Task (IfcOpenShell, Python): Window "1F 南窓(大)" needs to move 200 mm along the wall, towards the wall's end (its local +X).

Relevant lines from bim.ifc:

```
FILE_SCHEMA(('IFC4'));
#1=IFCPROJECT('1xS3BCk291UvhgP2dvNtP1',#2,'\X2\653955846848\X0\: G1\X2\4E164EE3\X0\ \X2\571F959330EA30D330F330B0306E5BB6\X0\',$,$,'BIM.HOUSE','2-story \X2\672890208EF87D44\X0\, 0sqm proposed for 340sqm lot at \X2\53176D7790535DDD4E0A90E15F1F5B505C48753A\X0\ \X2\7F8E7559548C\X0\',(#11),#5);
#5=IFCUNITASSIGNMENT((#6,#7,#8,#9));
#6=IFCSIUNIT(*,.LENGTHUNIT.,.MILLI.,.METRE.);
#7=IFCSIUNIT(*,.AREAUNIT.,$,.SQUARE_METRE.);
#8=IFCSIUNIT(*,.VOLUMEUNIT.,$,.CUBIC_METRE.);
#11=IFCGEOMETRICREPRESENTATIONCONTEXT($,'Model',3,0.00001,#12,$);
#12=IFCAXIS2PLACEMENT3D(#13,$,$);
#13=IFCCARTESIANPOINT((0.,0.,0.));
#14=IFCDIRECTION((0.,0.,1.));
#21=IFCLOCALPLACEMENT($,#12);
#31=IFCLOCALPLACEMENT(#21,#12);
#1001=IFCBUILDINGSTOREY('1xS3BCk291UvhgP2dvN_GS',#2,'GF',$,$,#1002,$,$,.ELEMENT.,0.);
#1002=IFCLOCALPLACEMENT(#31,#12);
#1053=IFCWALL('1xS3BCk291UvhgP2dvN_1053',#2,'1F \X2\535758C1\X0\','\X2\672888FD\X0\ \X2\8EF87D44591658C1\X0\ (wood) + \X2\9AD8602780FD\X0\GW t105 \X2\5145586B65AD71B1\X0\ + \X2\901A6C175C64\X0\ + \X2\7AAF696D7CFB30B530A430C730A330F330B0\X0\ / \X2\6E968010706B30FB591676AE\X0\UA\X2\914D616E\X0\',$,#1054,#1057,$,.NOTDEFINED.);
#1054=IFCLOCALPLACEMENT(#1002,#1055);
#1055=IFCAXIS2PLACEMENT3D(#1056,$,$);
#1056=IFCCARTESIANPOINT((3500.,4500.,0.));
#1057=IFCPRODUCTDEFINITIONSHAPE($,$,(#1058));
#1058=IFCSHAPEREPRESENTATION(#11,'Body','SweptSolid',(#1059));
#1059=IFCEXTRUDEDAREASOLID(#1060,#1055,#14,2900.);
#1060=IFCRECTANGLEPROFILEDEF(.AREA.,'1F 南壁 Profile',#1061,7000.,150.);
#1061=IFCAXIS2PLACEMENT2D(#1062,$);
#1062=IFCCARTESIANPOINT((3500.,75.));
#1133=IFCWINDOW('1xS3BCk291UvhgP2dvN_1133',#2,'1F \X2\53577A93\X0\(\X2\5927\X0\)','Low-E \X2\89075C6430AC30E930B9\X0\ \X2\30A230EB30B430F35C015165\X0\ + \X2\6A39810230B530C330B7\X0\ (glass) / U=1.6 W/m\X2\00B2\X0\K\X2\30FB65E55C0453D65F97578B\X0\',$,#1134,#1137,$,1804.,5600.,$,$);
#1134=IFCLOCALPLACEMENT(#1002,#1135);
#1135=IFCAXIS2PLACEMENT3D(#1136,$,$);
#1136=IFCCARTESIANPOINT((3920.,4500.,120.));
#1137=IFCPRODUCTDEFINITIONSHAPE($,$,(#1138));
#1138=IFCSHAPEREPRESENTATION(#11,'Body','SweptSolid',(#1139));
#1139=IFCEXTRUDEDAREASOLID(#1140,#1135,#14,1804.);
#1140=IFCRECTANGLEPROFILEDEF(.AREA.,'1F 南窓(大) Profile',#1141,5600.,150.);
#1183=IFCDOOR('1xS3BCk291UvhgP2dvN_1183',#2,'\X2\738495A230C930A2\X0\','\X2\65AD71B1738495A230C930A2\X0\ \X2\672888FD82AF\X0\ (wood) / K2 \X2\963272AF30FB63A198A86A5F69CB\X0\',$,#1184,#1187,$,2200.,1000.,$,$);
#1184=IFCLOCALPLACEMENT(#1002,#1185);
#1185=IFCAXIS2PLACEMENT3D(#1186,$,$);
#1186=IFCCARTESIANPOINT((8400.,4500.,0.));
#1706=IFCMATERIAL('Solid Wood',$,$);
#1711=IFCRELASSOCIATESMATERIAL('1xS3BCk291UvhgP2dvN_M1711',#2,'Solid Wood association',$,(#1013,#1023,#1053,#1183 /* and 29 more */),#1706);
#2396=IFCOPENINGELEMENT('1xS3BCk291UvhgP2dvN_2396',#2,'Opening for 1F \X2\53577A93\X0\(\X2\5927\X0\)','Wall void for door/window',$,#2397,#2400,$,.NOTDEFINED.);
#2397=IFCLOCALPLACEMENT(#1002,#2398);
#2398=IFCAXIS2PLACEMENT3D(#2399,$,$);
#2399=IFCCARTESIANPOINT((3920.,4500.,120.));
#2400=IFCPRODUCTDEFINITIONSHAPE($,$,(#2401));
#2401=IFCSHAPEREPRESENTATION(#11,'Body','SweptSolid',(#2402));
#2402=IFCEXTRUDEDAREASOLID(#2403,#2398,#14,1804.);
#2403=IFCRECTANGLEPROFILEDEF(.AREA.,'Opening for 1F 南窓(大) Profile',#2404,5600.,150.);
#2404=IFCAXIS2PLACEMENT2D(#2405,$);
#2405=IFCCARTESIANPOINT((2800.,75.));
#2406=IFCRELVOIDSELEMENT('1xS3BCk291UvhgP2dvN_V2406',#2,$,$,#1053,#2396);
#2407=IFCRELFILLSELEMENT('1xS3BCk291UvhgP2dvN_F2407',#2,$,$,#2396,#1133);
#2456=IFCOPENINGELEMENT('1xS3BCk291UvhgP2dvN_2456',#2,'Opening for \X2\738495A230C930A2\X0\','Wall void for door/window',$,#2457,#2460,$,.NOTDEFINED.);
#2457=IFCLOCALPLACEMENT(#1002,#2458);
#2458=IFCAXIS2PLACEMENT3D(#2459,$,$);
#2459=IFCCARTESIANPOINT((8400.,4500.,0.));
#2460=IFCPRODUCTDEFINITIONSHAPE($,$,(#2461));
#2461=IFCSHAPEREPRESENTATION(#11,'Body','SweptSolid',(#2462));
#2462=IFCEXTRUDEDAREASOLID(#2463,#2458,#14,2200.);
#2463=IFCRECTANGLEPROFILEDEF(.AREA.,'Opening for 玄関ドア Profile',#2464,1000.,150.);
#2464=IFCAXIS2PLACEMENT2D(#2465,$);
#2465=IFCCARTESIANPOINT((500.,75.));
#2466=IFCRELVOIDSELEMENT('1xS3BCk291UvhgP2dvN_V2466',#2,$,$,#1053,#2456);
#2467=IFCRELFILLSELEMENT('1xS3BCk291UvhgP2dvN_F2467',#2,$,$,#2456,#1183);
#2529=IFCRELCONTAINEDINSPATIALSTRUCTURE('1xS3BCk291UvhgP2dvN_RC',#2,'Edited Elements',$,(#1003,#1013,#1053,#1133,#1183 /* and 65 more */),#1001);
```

```python
import ifcopenshell
import ifcopenshell.api.geometry
import ifcopenshell.util.placement

model = ifcopenshell.open("bim.ifc")

window = model.by_guid("1xS3BCk291UvhgP2dvN_1133")
opening = window.FillsVoids[0].RelatingOpeningElement
wall = opening.VoidsElements[0].RelatingBuildingElement

wall_matrix = ifcopenshell.util.placement.get_local_placement(wall.ObjectPlacement)
shift = wall_matrix[:3, 0] * 200.0
before = ifcopenshell.util.placement.get_local_placement(window.ObjectPlacement)[:3, 3].copy()

# The window is not placed relative to its opening, so move both.
for product in (opening, window):
    matrix = ifcopenshell.util.placement.get_local_placement(product.ObjectPlacement)
    matrix[:3, 3] += shift
    ifcopenshell.api.geometry.edit_object_placement(model, product=product, matrix=matrix, is_si=False)

after = ifcopenshell.util.placement.get_local_placement(window.ObjectPlacement)[:3, 3]
print("window moved by", (after - before).round(3) + 0.0)

model.write("bim_v2.ifc")
```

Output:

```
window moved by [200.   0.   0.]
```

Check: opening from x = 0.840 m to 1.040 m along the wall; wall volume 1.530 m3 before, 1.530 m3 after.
